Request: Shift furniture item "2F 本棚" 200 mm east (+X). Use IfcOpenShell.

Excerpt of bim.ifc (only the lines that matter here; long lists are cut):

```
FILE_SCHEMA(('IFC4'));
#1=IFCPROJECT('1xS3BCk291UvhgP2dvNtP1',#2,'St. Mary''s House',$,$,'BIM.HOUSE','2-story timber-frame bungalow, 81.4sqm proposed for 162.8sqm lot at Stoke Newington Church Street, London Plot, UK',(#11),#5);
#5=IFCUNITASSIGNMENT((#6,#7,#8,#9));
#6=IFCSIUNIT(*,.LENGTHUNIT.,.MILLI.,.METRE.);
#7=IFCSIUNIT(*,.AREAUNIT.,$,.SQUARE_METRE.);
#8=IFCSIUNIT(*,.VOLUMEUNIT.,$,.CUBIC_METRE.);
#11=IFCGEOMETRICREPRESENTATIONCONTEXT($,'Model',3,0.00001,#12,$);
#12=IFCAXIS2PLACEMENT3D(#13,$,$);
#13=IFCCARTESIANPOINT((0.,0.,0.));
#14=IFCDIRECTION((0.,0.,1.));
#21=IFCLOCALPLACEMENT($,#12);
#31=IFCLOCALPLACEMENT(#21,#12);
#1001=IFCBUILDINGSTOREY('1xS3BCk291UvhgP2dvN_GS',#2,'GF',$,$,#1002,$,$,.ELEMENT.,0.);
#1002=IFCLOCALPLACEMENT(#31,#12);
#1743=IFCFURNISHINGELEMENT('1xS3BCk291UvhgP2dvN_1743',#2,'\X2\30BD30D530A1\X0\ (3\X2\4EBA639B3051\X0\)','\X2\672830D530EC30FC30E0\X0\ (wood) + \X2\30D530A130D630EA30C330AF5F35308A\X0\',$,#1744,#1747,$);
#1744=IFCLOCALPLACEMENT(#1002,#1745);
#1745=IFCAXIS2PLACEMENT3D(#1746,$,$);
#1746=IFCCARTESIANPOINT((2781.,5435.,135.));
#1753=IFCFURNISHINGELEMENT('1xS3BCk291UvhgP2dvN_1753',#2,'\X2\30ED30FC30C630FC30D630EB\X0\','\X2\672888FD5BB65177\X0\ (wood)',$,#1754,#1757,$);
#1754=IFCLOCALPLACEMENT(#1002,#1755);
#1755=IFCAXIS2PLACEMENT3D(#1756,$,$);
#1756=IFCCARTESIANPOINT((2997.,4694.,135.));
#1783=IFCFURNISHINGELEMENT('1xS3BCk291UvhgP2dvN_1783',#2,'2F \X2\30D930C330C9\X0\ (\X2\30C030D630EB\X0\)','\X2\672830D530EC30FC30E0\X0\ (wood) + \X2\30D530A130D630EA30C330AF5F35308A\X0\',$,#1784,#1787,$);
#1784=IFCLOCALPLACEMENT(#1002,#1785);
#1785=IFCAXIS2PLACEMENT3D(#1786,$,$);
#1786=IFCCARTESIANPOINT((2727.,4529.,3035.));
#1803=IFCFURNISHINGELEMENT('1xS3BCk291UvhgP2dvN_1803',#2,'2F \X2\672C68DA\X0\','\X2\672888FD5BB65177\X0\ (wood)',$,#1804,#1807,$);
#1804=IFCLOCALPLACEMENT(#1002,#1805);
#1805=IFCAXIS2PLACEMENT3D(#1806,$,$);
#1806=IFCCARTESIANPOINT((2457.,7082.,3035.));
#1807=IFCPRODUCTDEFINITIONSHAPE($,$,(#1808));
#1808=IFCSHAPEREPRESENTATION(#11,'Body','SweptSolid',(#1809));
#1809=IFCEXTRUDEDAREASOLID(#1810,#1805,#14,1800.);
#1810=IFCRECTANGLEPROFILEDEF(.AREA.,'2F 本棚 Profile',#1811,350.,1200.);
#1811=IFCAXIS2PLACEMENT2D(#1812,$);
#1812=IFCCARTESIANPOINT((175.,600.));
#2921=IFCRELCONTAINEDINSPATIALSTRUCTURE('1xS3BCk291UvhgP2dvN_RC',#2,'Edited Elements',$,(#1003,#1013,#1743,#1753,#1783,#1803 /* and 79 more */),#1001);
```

```python
import ifcopenshell
import ifcopenshell.api.geometry
import ifcopenshell.util.placement
import ifcopenshell.util.unit

model = ifcopenshell.open("bim.ifc")
unit_scale = ifcopenshell.util.unit.calculate_unit_scale(model)

item = model.by_guid("1xS3BCk291UvhgP2dvN_1803")
matrix = ifcopenshell.util.placement.get_local_placement(item.ObjectPlacement)
matrix[0, 3] += 0.2 / unit_scale
ifcopenshell.api.geometry.edit_object_placement(model, product=item, matrix=matrix, is_si=False)

print(ifcopenshell.util.placement.get_local_placement(item.ObjectPlacement).round(3) + 0.0)

model.write("bim-out.ifc")
```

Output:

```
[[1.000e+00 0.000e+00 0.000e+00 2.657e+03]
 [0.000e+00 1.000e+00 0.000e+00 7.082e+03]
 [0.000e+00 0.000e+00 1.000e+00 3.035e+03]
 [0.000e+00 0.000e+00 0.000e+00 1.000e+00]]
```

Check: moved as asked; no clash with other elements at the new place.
